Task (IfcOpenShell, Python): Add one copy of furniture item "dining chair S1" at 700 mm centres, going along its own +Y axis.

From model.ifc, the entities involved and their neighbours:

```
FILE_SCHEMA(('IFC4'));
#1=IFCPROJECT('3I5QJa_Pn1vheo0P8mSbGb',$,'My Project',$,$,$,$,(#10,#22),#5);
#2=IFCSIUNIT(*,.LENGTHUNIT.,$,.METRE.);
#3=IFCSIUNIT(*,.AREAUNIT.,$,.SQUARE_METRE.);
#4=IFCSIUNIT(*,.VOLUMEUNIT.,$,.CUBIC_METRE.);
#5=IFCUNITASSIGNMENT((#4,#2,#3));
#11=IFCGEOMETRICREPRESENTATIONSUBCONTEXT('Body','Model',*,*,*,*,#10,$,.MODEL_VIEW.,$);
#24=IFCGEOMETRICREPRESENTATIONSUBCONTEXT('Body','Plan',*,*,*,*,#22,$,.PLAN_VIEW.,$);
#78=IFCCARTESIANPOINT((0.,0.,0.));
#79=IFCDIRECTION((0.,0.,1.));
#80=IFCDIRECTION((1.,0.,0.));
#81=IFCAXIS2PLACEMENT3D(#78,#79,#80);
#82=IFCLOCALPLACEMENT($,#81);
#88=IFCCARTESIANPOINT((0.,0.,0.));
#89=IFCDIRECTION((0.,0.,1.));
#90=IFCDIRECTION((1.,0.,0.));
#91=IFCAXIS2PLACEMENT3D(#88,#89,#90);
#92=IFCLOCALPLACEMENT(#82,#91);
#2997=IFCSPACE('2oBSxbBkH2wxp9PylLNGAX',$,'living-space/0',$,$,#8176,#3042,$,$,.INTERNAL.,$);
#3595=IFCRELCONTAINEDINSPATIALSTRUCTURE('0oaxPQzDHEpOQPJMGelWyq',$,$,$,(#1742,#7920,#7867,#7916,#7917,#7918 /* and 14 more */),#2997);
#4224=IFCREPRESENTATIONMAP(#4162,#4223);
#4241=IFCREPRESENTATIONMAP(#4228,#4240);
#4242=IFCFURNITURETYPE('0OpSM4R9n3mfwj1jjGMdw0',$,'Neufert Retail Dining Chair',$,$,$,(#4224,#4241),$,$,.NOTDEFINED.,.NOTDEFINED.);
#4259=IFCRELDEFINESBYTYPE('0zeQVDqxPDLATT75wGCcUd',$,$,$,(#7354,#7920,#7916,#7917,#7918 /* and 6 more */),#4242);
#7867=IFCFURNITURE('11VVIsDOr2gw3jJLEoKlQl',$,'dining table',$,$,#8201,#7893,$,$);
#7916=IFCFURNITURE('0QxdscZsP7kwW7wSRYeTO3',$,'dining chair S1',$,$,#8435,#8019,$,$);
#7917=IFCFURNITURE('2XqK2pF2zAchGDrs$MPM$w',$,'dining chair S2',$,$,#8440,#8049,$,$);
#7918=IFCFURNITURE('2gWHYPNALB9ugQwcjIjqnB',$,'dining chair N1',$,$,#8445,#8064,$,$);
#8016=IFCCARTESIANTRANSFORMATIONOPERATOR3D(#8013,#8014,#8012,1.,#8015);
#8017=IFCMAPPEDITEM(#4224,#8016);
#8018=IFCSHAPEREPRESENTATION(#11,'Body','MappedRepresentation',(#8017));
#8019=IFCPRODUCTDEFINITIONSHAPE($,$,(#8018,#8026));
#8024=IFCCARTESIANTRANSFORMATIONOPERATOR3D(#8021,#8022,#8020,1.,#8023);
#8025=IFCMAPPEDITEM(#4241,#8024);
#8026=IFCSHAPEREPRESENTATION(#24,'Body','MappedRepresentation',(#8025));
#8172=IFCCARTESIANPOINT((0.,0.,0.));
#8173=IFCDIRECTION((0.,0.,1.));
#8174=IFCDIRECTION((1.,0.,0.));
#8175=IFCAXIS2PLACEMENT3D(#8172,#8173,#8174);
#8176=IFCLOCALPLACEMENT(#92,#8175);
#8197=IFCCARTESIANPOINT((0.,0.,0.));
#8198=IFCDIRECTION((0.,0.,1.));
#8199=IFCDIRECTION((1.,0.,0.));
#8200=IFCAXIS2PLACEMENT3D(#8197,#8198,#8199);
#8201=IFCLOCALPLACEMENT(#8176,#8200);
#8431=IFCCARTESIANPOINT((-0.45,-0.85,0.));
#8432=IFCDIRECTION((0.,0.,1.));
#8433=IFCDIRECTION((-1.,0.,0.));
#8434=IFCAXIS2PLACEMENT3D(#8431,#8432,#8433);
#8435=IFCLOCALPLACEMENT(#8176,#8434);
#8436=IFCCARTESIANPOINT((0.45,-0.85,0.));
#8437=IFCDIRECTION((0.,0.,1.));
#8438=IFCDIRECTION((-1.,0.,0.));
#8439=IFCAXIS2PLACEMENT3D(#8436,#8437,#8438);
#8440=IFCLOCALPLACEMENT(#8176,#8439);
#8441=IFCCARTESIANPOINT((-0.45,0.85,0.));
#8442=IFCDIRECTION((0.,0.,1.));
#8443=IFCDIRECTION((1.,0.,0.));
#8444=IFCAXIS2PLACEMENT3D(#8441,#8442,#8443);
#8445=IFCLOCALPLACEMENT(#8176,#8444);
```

```python
import ifcopenshell
import ifcopenshell.api.geometry
import ifcopenshell.api.root
import ifcopenshell.util.element
import ifcopenshell.util.placement

model = ifcopenshell.open("model.ifc")

source = model.by_guid("0QxdscZsP7kwW7wSRYeTO3")
base = ifcopenshell.util.placement.get_local_placement(source.ObjectPlacement)
step = base[:3, 1] * 0.7

for i in range(1, 2):
    copy = ifcopenshell.api.root.copy_class(model, product=source)
    copy.Representation = ifcopenshell.util.element.copy_deep(
        model, source.Representation, exclude=["IfcGeometricRepresentationContext", "IfcRepresentationMap"]
    )
    matrix = base.copy()
    matrix[:3, 3] += i * step
    print("added at", matrix[:3, 3].round(3) + 0.0)
    ifcopenshell.api.geometry.edit_object_placement(model, product=copy, matrix=matrix, is_si=False)

model.write("model_updated.ifc")
```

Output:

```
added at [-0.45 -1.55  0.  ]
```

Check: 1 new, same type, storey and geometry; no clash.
